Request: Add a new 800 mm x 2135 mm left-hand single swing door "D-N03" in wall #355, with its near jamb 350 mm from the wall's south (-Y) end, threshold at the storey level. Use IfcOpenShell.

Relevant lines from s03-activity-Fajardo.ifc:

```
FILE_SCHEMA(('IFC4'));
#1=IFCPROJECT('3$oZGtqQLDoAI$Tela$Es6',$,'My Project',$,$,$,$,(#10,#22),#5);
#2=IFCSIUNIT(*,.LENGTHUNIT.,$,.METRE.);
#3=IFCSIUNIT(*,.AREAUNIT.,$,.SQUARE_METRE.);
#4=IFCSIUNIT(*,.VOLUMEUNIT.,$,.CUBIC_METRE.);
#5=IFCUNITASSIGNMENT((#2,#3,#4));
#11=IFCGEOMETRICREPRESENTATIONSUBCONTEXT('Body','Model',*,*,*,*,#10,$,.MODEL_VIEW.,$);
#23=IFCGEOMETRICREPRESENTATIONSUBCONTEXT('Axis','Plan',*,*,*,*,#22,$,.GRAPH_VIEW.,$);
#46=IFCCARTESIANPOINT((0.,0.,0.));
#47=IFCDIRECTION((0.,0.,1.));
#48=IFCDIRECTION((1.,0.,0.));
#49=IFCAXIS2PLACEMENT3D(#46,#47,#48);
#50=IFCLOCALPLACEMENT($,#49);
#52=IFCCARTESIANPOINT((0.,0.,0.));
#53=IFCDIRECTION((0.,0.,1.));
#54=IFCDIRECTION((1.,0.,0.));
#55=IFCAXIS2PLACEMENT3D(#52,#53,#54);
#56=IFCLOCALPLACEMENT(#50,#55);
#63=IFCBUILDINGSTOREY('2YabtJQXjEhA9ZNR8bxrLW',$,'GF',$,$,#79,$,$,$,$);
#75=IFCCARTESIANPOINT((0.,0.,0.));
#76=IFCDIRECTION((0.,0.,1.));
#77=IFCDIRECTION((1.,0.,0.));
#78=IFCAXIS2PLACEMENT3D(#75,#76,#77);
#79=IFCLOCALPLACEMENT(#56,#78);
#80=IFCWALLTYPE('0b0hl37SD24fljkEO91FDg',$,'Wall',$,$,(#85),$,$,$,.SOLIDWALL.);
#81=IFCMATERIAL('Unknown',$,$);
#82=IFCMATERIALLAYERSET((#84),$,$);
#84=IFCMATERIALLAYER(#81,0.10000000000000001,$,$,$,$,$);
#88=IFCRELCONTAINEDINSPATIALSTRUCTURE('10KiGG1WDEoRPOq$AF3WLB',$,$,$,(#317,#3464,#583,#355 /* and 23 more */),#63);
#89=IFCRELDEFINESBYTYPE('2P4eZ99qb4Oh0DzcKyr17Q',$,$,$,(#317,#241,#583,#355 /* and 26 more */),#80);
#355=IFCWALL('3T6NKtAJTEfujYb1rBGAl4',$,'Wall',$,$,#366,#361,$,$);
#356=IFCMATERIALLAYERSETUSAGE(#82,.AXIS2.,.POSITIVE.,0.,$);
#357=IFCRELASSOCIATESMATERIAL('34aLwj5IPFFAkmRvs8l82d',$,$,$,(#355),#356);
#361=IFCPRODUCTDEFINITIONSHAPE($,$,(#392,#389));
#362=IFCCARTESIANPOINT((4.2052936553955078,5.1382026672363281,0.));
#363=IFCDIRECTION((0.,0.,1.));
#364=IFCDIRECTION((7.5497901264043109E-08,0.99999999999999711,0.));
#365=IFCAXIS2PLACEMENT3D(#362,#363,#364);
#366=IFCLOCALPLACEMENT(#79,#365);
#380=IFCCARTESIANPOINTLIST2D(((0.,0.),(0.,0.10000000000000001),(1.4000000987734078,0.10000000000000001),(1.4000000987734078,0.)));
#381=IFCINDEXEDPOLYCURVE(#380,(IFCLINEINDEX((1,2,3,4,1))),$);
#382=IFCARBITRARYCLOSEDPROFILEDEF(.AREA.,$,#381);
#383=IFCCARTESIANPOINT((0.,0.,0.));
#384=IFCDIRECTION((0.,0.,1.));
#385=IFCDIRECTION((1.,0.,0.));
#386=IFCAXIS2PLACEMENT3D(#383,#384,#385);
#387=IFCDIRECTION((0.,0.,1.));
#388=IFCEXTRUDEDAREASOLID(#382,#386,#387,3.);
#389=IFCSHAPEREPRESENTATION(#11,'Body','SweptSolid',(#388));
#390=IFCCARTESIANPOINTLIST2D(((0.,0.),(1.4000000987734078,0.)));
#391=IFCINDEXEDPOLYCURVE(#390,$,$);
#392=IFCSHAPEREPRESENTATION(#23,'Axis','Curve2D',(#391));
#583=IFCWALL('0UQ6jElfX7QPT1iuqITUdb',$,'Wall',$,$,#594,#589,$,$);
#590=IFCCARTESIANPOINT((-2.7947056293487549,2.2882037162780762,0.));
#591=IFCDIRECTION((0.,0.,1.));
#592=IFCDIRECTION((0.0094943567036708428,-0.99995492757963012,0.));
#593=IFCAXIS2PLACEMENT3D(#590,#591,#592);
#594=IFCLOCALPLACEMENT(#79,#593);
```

```python
import numpy as np
import ifcopenshell
import ifcopenshell.api.feature
import ifcopenshell.api.geometry
import ifcopenshell.api.root
import ifcopenshell.api.spatial
import ifcopenshell.geom
import ifcopenshell.util.element
import ifcopenshell.util.placement
import ifcopenshell.util.representation
import ifcopenshell.util.shape
import ifcopenshell.util.unit

model = ifcopenshell.open("s03-activity-Fajardo.ifc")
unit_scale = ifcopenshell.util.unit.calculate_unit_scale(model)
settings = ifcopenshell.geom.settings()


def volume(element):
    """Net volume in cubic metres, openings subtracted."""
    shape = ifcopenshell.geom.create_shape(settings, element)
    return ifcopenshell.util.shape.get_volume(shape.geometry)


wall = model.by_guid("3T6NKtAJTEfujYb1rBGAl4")
storey = ifcopenshell.util.element.get_container(wall, ifc_class="IfcBuildingStorey")
context = ifcopenshell.util.representation.get_context(model, "Model", "Body", "MODEL_VIEW")
before = volume(wall)

width, height, from_end, sill = 0.8, 2.135, 0.35, 0.0  # metres

# The wall runs along its own X axis, and the end named is its -X end.
wall_shape = ifcopenshell.geom.create_shape(settings, wall)
x, y, z = ifcopenshell.util.shape.get_vertices(wall_shape.geometry).T
start = x.min() + from_end
face, thickness = float(y.min()), float(y.max() - y.min())
wall_matrix = ifcopenshell.util.placement.get_local_placement(wall.ObjectPlacement)
level = ifcopenshell.util.placement.get_local_placement(storey.ObjectPlacement)[2, 3]


def in_wall(x, y):
    """Placement at x, y metres in the wall's axes, at sill height."""
    matrix = wall_matrix.copy()
    matrix[:, 3] = wall_matrix @ np.array([x / unit_scale, y / unit_scale, 0.0, 1.0])
    matrix[2, 3] = level + sill / unit_scale
    return matrix


# Opening: a box that overshoots both wall faces by 50 mm.
opening = ifcopenshell.api.root.create_entity(model, ifc_class="IfcOpeningElement", predefined_type="OPENING")
box = ifcopenshell.api.geometry.add_wall_representation(
    model, context=context, length=width, height=height, thickness=thickness + 0.1
)
ifcopenshell.api.geometry.assign_representation(model, product=opening, representation=box)
ifcopenshell.api.geometry.edit_object_placement(model, product=opening, matrix=in_wall(start, face - 0.05), is_si=False)
ifcopenshell.api.feature.add_feature(model, feature=opening, element=wall)

door = ifcopenshell.api.root.create_entity(model, ifc_class="IfcDoor", name="D-N03", predefined_type="DOOR")
door.OverallWidth, door.OverallHeight = width / unit_scale, height / unit_scale
door.OperationType = "SINGLE_SWING_LEFT"
body = ifcopenshell.api.geometry.add_door_representation(
    model,
    context=context,
    overall_width=door.OverallWidth,
    overall_height=door.OverallHeight,
    operation_type="SINGLE_SWING_LEFT",
    lining_properties={"LiningDepth": thickness / unit_scale, "ThresholdDepth": thickness / unit_scale},
)
ifcopenshell.api.geometry.assign_representation(model, product=door, representation=body)
ifcopenshell.api.spatial.assign_container(model, products=[door], relating_structure=storey)
ifcopenshell.api.feature.add_filling(model, opening=opening, element=door)

# The lining spans the wall, so the door starts at the wall face.
ifcopenshell.api.geometry.edit_object_placement(model, product=door, matrix=in_wall(start, face), is_si=False)

after = volume(wall)

print(f"wall volume {before:.3f} -> {after:.3f} m3")

model.write("s03-activity-Fajardo_v2.ifc")
```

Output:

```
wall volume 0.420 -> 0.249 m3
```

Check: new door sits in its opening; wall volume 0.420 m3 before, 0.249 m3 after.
